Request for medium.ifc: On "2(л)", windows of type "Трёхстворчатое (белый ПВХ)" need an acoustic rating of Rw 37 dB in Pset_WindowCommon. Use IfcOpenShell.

First a look at what the model holds.

```python
import ifcopenshell
import ifcopenshell.util.element

model = ifcopenshell.open("medium.ifc")
print(model.schema)
storey = next(s for s in model.by_type("IfcBuildingStorey") if s.Name == "2(л)")
windows = [e for e in ifcopenshell.util.element.get_decomposition(storey) if e.is_a("IfcWindow")]
seen = {}
for e in windows:
    element_type = ifcopenshell.util.element.get_type(e)
    key = (element_type.Name if element_type != e and element_type else None, ifcopenshell.util.element.get_pset(e, "Pset_WindowCommon", "AcousticRating"))
    seen[key] = seen.get(key, 0) + 1
for (name, value), count in sorted(seen.items(), key=str):
    print(count, "x", name, "|", value)
```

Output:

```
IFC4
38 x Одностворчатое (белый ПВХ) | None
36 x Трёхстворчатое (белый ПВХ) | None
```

```python
import ifcopenshell
import ifcopenshell.api.pset
import ifcopenshell.util.element

model = ifcopenshell.open("medium.ifc")

storey = next(s for s in model.by_type("IfcBuildingStorey") if s.Name == "2(л)")
windows = [e for e in ifcopenshell.util.element.get_decomposition(storey) if e.is_a("IfcWindow")]

count = 0
for e in windows:
    element_type = ifcopenshell.util.element.get_type(e)
    if element_type in (None, e) or element_type.Name != "Трёхстворчатое (белый ПВХ)":
        continue
    # add_pset returns the element's existing set when there is one.
    pset = ifcopenshell.api.pset.add_pset(model, product=e, name="Pset_WindowCommon")
    ifcopenshell.api.pset.edit_pset(model, pset=pset, properties={"AcousticRating": "Rw 37 dB"})
    count += 1

print(count, "windows updated")

model.write("medium_edited.ifc")
```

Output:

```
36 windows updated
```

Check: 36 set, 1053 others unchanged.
